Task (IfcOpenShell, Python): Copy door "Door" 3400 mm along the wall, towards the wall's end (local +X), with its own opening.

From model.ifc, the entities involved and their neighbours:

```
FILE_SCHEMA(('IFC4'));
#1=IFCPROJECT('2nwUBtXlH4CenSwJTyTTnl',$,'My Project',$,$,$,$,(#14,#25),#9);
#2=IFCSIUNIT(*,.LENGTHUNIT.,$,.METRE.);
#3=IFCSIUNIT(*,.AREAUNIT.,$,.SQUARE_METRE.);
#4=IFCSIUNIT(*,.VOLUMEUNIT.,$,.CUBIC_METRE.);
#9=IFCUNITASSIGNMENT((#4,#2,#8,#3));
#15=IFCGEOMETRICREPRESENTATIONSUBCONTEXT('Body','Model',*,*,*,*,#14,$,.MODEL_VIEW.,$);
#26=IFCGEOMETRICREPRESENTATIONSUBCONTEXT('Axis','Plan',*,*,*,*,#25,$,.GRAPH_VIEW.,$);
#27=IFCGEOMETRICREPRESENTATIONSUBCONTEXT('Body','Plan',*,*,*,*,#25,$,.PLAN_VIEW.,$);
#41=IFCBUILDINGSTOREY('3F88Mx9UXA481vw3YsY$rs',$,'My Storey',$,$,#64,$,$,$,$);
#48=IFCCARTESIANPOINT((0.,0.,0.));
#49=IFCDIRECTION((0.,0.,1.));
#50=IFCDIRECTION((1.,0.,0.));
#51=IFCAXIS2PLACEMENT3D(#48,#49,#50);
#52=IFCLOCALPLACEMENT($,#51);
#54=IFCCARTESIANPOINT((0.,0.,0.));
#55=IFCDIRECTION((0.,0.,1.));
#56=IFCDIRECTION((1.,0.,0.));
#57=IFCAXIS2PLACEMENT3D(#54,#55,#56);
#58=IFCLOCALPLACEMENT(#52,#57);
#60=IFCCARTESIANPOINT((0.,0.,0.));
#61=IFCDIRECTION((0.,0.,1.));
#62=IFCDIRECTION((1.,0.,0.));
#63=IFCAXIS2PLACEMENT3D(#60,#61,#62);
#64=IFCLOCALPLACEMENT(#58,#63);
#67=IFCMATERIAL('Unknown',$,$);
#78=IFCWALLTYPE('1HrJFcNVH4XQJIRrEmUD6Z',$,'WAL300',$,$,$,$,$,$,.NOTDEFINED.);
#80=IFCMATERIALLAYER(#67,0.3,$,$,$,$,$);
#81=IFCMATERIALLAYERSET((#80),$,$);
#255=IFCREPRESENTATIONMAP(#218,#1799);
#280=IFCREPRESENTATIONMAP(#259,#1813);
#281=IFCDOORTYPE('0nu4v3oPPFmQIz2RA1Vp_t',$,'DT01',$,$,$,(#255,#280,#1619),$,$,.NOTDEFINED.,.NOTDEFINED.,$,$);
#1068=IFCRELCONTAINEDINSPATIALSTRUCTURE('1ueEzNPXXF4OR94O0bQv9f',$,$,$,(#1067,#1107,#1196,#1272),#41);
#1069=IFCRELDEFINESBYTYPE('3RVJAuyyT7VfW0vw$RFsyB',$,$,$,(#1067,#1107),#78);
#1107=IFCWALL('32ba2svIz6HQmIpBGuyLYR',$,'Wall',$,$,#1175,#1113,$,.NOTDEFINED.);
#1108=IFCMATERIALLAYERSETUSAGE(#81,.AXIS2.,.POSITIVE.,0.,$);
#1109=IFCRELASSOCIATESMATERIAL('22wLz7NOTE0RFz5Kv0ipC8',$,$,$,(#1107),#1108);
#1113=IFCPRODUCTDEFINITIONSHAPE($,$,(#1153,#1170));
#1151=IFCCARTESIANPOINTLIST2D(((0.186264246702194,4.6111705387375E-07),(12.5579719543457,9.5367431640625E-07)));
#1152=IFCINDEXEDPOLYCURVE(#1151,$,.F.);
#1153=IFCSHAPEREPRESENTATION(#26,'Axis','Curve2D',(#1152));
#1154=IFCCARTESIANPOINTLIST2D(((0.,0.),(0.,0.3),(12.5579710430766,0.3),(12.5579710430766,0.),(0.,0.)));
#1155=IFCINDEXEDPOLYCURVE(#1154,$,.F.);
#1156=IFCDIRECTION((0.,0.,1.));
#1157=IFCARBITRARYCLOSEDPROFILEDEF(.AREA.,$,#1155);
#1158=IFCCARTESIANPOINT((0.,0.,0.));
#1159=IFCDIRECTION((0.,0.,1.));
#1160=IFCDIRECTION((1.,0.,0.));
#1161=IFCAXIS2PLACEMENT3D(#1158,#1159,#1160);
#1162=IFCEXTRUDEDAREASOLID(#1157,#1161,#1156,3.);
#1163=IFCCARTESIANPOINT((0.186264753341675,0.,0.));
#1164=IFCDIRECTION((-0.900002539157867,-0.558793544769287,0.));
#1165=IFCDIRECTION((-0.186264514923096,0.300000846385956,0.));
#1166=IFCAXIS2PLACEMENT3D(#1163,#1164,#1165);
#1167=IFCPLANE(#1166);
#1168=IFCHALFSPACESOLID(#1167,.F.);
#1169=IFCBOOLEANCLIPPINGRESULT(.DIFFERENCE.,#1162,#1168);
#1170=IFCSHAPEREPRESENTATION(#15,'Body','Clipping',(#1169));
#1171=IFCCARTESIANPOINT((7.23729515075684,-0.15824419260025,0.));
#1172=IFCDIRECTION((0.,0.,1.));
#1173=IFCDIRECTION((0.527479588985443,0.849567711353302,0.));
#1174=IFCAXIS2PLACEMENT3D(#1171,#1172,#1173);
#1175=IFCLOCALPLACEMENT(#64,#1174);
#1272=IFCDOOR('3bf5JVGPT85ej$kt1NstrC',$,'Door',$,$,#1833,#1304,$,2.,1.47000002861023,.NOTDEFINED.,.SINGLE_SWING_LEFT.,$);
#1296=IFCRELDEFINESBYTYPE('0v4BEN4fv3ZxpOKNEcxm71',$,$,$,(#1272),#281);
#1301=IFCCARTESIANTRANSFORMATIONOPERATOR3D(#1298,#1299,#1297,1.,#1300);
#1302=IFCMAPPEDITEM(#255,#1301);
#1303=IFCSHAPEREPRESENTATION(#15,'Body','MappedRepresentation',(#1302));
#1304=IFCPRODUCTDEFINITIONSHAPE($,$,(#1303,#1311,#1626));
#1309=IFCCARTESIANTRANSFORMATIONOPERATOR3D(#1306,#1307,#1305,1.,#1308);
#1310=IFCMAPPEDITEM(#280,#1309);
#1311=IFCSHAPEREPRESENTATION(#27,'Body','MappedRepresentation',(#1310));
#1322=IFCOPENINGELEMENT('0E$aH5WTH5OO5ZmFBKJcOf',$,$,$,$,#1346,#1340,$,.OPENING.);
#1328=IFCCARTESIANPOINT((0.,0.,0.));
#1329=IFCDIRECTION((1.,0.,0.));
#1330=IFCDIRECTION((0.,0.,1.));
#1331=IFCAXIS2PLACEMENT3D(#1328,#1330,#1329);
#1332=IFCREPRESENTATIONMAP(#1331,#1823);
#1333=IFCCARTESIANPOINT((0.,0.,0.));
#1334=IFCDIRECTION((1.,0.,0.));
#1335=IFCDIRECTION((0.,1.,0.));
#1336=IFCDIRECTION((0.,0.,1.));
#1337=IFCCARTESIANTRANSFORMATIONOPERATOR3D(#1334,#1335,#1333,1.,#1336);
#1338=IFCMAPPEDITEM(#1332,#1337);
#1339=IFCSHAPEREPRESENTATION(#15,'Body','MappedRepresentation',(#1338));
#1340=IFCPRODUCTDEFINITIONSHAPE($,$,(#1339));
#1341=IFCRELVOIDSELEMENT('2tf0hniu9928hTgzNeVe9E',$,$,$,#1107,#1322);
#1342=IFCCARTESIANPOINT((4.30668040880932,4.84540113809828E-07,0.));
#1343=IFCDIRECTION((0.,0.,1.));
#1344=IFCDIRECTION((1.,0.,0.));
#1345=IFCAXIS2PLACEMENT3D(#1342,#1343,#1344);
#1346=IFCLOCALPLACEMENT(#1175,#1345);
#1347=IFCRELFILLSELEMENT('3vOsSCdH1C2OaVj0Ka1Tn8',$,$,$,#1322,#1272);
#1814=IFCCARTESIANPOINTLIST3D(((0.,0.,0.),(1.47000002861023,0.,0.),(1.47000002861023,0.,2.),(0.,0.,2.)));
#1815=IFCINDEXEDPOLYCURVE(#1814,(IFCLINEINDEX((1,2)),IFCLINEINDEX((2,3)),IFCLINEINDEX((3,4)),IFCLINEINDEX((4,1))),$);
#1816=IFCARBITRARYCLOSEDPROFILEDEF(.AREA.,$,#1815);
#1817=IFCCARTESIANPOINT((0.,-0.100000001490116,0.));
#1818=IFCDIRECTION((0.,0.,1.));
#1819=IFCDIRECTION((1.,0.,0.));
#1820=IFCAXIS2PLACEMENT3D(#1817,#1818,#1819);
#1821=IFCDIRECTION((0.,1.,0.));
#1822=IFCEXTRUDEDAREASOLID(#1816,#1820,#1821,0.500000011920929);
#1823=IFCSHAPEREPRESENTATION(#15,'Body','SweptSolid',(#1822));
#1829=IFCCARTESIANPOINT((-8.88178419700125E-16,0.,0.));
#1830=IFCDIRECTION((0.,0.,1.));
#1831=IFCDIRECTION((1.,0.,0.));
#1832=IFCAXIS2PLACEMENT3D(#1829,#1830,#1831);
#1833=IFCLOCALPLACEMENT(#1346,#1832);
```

```python
import ifcopenshell
import ifcopenshell.api.feature
import ifcopenshell.api.geometry
import ifcopenshell.api.root
import ifcopenshell.geom
import ifcopenshell.util.element
import ifcopenshell.util.placement
import ifcopenshell.util.shape
import ifcopenshell.util.unit

model = ifcopenshell.open("model.ifc")
unit_scale = ifcopenshell.util.unit.calculate_unit_scale(model)
settings = ifcopenshell.geom.settings()


def volume(element):
    """Net volume in cubic metres, openings subtracted."""
    shape = ifcopenshell.geom.create_shape(settings, element)
    return ifcopenshell.util.shape.get_volume(shape.geometry)


door = model.by_id(1272)
opening = door.FillsVoids[0].RelatingOpeningElement
wall = opening.VoidsElements[0].RelatingBuildingElement
before = volume(wall)
shift = ifcopenshell.util.placement.get_local_placement(wall.ObjectPlacement)[:3, 0] * 3.4 / unit_scale

# copy_class copies the void relationship, type, container and properties, but no geometry.
new_opening = ifcopenshell.api.root.copy_class(model, product=opening)
new_opening.Representation = ifcopenshell.util.element.copy_deep(
    model, opening.Representation, exclude=["IfcGeometricRepresentationContext", "IfcRepresentationMap"]
)
new_door = ifcopenshell.api.root.copy_class(model, product=door)
new_door.Representation = ifcopenshell.util.element.copy_deep(
    model, door.Representation, exclude=["IfcGeometricRepresentationContext", "IfcRepresentationMap"]
)
ifcopenshell.api.feature.add_filling(model, opening=new_opening, element=new_door)

for old, new in ((opening, new_opening), (door, new_door)):
    matrix = ifcopenshell.util.placement.get_local_placement(old.ObjectPlacement)
    matrix[:3, 3] += shift
    ifcopenshell.api.geometry.edit_object_placement(model, product=new, matrix=matrix, is_si=False)

after = volume(wall)

print(f"wall volume {before:.3f} -> {after:.3f} m3")

model.write("model_updated.ifc")
```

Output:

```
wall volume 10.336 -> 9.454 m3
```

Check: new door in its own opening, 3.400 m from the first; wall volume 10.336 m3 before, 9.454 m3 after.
